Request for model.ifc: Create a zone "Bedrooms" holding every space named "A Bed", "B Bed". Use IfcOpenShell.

First a look at what the model holds.

```python
import ifcopenshell

model = ifcopenshell.open("model.ifc")
print(model.schema)
seen = {}
for space in model.by_type("IfcSpace"):
    seen[space.Name] = seen.get(space.Name, 0) + 1
for name, count in sorted(seen.items(), key=str):
    print(count, "x", name)
print("zones:", [z.Name for z in model.by_type("IfcZone")][:20])
```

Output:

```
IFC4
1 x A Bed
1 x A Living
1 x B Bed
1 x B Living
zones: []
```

```python
import ifcopenshell
import ifcopenshell.api.group
import ifcopenshell.api.root

model = ifcopenshell.open("model.ifc")

names = {"A Bed", "B Bed"}
spaces = [s for s in model.by_type("IfcSpace") if s.Name in names]

zone = ifcopenshell.api.root.create_entity(model, ifc_class="IfcZone", name="Bedrooms")
ifcopenshell.api.group.assign_group(model, products=spaces, group=zone)
print(len(spaces), "spaces in", zone.Name)

model.write("model-out.ifc")
```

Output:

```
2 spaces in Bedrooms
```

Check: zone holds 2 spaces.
